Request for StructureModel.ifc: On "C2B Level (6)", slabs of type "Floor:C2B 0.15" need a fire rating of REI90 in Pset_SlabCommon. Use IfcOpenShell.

First a look at what the model holds.

```python
import ifcopenshell
import ifcopenshell.util.element

model = ifcopenshell.open("StructureModel.ifc")
print(model.schema)
storey = next(s for s in model.by_type("IfcBuildingStorey") if s.Name == "C2B Level (6)")
slabs = [e for e in ifcopenshell.util.element.get_decomposition(storey) if e.is_a("IfcSlab")]
seen = {}
for e in slabs:
    element_type = ifcopenshell.util.element.get_type(e)
    key = (element_type.Name if element_type != e and element_type else None, ifcopenshell.util.element.get_pset(e, "Pset_SlabCommon", "FireRating"))
    seen[key] = seen.get(key, 0) + 1
for (name, value), count in sorted(seen.items(), key=str):
    print(count, "x", name, "|", value)
```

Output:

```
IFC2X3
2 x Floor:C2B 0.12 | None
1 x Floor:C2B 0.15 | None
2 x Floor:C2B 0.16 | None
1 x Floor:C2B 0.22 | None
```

```python
import ifcopenshell
import ifcopenshell.api.pset
import ifcopenshell.util.element

model = ifcopenshell.open("StructureModel.ifc")

storey = next(s for s in model.by_type("IfcBuildingStorey") if s.Name == "C2B Level (6)")
slabs = [e for e in ifcopenshell.util.element.get_decomposition(storey) if e.is_a("IfcSlab")]

count = 0
for e in slabs:
    element_type = ifcopenshell.util.element.get_type(e)
    if element_type in (None, e) or element_type.Name != "Floor:C2B 0.15":
        continue
    # add_pset returns the element's existing set when there is one.
    pset = ifcopenshell.api.pset.add_pset(model, product=e, name="Pset_SlabCommon")
    ifcopenshell.api.pset.edit_pset(model, pset=pset, properties={"FireRating": "REI90"})
    count += 1

print(count, "slabs updated")

model.write("StructureModel_v2.ifc")
```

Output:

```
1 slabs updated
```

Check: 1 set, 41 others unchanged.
